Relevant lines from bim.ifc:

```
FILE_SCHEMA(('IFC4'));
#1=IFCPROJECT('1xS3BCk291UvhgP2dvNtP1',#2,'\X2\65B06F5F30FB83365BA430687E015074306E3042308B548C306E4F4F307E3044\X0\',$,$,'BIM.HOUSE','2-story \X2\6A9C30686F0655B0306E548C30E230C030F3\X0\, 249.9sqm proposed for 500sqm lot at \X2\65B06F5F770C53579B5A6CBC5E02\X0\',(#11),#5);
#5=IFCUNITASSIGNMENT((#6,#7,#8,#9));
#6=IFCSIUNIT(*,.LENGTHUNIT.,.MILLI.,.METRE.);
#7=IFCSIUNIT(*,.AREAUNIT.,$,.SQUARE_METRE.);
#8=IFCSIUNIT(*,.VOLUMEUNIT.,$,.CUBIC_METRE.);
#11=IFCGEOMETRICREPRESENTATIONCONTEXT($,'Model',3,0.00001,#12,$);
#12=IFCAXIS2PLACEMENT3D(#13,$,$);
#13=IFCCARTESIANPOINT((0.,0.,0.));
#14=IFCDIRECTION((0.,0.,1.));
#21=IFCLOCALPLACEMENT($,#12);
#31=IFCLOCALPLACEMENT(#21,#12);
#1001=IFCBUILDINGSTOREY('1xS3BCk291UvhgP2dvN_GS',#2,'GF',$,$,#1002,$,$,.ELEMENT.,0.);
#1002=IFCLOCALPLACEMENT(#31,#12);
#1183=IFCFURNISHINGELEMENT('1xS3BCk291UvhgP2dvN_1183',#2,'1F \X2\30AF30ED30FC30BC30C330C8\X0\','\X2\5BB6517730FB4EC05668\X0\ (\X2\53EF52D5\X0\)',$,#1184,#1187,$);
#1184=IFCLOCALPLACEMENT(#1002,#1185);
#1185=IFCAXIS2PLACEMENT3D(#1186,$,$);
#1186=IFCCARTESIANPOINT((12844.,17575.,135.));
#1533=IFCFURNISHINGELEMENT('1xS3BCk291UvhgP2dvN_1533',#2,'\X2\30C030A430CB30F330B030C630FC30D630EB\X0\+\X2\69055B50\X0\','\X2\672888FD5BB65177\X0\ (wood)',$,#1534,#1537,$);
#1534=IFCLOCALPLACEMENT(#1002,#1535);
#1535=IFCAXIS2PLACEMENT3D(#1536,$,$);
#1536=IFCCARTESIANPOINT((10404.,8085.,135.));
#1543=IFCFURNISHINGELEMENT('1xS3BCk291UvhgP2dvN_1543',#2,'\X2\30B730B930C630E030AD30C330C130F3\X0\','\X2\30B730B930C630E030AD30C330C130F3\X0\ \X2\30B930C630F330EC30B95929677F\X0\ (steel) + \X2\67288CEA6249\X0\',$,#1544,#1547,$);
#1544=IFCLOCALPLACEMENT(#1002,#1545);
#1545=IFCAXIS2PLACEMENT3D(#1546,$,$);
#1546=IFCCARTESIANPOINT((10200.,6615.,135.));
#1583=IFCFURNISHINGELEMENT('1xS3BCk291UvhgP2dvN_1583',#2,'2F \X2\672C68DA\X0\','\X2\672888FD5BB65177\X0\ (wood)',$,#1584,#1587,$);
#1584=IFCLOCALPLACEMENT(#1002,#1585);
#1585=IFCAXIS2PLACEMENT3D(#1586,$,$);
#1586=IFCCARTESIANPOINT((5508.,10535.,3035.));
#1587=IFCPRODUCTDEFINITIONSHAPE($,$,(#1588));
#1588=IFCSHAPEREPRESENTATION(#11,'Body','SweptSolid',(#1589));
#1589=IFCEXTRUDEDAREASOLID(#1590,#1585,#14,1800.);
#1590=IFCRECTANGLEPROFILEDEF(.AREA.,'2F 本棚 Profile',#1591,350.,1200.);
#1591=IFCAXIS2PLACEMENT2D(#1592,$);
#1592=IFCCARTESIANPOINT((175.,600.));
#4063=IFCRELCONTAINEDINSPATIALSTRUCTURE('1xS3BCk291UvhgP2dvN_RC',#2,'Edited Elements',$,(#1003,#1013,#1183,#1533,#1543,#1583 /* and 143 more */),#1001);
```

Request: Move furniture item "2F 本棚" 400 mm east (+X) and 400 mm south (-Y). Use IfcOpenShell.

```python
import ifcopenshell
import ifcopenshell.api.geometry
import ifcopenshell.util.placement
import ifcopenshell.util.unit

model = ifcopenshell.open("bim.ifc")
unit_scale = ifcopenshell.util.unit.calculate_unit_scale(model)

item = model.by_guid("1xS3BCk291UvhgP2dvN_1583")
matrix = ifcopenshell.util.placement.get_local_placement(item.ObjectPlacement)
matrix[0, 3] += 0.4 / unit_scale
matrix[1, 3] -= 0.4 / unit_scale
ifcopenshell.api.geometry.edit_object_placement(model, product=item, matrix=matrix, is_si=False)

print(ifcopenshell.util.placement.get_local_placement(item.ObjectPlacement).round(3) + 0.0)

model.write("bim_edited.ifc")
```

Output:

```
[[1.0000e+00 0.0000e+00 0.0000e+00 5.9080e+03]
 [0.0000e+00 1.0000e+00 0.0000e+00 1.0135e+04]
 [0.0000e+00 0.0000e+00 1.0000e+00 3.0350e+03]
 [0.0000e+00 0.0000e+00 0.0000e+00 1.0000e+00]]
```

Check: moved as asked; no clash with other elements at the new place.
